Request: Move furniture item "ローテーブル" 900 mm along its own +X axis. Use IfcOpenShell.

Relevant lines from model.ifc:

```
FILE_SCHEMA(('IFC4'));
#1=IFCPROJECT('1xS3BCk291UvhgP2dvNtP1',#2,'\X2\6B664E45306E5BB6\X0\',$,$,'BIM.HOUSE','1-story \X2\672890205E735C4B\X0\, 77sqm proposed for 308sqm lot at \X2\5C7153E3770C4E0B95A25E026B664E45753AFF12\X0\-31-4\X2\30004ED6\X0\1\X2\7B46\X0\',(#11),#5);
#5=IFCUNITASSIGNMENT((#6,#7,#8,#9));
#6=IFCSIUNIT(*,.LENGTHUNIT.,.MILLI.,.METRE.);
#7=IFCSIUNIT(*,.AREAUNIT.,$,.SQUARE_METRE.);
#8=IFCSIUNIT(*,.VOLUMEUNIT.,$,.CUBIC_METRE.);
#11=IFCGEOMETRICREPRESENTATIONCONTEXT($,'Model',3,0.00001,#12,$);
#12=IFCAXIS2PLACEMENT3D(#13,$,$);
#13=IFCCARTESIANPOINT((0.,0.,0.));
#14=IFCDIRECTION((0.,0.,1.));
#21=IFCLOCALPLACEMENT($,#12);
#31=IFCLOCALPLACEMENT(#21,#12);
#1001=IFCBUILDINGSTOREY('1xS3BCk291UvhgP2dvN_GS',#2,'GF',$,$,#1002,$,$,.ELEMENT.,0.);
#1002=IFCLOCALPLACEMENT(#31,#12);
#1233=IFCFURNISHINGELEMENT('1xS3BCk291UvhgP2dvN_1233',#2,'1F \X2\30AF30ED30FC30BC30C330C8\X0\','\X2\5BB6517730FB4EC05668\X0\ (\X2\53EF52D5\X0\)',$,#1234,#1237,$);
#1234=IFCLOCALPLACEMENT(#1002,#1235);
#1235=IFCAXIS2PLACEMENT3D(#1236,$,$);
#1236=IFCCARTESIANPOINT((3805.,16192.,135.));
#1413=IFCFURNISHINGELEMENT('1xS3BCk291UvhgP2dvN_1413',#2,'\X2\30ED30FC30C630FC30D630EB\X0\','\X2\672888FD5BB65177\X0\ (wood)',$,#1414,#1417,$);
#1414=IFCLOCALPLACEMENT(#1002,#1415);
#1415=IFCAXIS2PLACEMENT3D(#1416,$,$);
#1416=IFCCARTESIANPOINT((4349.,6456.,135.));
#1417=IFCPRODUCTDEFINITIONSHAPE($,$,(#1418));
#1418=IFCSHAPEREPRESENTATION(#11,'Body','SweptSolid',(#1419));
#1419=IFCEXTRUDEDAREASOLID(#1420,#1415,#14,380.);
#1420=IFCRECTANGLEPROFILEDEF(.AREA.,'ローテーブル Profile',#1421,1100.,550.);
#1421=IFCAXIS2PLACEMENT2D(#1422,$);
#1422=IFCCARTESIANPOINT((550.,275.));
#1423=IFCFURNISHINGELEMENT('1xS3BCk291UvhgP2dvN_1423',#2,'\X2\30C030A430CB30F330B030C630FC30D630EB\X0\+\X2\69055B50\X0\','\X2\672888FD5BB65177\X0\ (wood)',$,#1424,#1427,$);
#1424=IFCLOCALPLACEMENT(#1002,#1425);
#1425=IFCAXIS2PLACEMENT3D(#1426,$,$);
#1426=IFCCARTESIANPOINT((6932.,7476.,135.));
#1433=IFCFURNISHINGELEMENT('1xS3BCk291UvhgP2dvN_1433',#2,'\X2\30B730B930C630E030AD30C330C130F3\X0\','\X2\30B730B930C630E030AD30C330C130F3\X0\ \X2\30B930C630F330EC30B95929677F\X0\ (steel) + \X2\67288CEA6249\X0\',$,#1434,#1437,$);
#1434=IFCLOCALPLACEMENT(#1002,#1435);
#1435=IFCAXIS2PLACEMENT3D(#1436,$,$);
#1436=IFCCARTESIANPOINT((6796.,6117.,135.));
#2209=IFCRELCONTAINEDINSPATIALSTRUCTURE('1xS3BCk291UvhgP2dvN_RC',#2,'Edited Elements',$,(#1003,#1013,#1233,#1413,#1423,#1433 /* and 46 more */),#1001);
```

```python
import ifcopenshell
import ifcopenshell.api.geometry
import ifcopenshell.util.placement
import ifcopenshell.util.unit

model = ifcopenshell.open("model.ifc")
unit_scale = ifcopenshell.util.unit.calculate_unit_scale(model)

item = model.by_guid("1xS3BCk291UvhgP2dvN_1413")
matrix = ifcopenshell.util.placement.get_local_placement(item.ObjectPlacement)
matrix[:3, 3] += matrix[:3, 0] * 0.9 / unit_scale
ifcopenshell.api.geometry.edit_object_placement(model, product=item, matrix=matrix, is_si=False)

print(ifcopenshell.util.placement.get_local_placement(item.ObjectPlacement).round(3) + 0.0)

model.write("model_edited.ifc")
```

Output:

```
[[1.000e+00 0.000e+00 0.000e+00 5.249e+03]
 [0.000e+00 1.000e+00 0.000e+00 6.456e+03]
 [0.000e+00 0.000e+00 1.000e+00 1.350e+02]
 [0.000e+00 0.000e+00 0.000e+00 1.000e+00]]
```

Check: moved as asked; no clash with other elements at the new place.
